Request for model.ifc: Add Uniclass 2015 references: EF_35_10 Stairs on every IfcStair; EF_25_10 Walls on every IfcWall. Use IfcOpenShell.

First a look at what the model holds.

```python
import ifcopenshell

model = ifcopenshell.open("model.ifc")
print(model.schema)
print("classifications:", [c.Name for c in model.by_type("IfcClassification")])
for ifc_class in ("IfcDoor", "IfcRoof", "IfcStair", "IfcWall", "IfcWindow"):
    print(ifc_class, len(model.by_type(ifc_class)))
```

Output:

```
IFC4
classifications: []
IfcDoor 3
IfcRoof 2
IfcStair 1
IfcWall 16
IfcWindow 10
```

```python
import ifcopenshell
import ifcopenshell.api.classification

model = ifcopenshell.open("model.ifc")

system = ifcopenshell.api.classification.add_classification(model, classification="Uniclass 2015")

codes = {
    "IfcStair": ("EF_35_10", "Stairs"),
    "IfcWall": ("EF_25_10", "Walls"),
}
for ifc_class, (code, name) in codes.items():
    products = model.by_type(ifc_class)
    ifcopenshell.api.classification.add_reference(
        model, products=products, classification=system, identification=code, name=name
    )
    print(code, len(products))

model.write("model_v2.ifc")
```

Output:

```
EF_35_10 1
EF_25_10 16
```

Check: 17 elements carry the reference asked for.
